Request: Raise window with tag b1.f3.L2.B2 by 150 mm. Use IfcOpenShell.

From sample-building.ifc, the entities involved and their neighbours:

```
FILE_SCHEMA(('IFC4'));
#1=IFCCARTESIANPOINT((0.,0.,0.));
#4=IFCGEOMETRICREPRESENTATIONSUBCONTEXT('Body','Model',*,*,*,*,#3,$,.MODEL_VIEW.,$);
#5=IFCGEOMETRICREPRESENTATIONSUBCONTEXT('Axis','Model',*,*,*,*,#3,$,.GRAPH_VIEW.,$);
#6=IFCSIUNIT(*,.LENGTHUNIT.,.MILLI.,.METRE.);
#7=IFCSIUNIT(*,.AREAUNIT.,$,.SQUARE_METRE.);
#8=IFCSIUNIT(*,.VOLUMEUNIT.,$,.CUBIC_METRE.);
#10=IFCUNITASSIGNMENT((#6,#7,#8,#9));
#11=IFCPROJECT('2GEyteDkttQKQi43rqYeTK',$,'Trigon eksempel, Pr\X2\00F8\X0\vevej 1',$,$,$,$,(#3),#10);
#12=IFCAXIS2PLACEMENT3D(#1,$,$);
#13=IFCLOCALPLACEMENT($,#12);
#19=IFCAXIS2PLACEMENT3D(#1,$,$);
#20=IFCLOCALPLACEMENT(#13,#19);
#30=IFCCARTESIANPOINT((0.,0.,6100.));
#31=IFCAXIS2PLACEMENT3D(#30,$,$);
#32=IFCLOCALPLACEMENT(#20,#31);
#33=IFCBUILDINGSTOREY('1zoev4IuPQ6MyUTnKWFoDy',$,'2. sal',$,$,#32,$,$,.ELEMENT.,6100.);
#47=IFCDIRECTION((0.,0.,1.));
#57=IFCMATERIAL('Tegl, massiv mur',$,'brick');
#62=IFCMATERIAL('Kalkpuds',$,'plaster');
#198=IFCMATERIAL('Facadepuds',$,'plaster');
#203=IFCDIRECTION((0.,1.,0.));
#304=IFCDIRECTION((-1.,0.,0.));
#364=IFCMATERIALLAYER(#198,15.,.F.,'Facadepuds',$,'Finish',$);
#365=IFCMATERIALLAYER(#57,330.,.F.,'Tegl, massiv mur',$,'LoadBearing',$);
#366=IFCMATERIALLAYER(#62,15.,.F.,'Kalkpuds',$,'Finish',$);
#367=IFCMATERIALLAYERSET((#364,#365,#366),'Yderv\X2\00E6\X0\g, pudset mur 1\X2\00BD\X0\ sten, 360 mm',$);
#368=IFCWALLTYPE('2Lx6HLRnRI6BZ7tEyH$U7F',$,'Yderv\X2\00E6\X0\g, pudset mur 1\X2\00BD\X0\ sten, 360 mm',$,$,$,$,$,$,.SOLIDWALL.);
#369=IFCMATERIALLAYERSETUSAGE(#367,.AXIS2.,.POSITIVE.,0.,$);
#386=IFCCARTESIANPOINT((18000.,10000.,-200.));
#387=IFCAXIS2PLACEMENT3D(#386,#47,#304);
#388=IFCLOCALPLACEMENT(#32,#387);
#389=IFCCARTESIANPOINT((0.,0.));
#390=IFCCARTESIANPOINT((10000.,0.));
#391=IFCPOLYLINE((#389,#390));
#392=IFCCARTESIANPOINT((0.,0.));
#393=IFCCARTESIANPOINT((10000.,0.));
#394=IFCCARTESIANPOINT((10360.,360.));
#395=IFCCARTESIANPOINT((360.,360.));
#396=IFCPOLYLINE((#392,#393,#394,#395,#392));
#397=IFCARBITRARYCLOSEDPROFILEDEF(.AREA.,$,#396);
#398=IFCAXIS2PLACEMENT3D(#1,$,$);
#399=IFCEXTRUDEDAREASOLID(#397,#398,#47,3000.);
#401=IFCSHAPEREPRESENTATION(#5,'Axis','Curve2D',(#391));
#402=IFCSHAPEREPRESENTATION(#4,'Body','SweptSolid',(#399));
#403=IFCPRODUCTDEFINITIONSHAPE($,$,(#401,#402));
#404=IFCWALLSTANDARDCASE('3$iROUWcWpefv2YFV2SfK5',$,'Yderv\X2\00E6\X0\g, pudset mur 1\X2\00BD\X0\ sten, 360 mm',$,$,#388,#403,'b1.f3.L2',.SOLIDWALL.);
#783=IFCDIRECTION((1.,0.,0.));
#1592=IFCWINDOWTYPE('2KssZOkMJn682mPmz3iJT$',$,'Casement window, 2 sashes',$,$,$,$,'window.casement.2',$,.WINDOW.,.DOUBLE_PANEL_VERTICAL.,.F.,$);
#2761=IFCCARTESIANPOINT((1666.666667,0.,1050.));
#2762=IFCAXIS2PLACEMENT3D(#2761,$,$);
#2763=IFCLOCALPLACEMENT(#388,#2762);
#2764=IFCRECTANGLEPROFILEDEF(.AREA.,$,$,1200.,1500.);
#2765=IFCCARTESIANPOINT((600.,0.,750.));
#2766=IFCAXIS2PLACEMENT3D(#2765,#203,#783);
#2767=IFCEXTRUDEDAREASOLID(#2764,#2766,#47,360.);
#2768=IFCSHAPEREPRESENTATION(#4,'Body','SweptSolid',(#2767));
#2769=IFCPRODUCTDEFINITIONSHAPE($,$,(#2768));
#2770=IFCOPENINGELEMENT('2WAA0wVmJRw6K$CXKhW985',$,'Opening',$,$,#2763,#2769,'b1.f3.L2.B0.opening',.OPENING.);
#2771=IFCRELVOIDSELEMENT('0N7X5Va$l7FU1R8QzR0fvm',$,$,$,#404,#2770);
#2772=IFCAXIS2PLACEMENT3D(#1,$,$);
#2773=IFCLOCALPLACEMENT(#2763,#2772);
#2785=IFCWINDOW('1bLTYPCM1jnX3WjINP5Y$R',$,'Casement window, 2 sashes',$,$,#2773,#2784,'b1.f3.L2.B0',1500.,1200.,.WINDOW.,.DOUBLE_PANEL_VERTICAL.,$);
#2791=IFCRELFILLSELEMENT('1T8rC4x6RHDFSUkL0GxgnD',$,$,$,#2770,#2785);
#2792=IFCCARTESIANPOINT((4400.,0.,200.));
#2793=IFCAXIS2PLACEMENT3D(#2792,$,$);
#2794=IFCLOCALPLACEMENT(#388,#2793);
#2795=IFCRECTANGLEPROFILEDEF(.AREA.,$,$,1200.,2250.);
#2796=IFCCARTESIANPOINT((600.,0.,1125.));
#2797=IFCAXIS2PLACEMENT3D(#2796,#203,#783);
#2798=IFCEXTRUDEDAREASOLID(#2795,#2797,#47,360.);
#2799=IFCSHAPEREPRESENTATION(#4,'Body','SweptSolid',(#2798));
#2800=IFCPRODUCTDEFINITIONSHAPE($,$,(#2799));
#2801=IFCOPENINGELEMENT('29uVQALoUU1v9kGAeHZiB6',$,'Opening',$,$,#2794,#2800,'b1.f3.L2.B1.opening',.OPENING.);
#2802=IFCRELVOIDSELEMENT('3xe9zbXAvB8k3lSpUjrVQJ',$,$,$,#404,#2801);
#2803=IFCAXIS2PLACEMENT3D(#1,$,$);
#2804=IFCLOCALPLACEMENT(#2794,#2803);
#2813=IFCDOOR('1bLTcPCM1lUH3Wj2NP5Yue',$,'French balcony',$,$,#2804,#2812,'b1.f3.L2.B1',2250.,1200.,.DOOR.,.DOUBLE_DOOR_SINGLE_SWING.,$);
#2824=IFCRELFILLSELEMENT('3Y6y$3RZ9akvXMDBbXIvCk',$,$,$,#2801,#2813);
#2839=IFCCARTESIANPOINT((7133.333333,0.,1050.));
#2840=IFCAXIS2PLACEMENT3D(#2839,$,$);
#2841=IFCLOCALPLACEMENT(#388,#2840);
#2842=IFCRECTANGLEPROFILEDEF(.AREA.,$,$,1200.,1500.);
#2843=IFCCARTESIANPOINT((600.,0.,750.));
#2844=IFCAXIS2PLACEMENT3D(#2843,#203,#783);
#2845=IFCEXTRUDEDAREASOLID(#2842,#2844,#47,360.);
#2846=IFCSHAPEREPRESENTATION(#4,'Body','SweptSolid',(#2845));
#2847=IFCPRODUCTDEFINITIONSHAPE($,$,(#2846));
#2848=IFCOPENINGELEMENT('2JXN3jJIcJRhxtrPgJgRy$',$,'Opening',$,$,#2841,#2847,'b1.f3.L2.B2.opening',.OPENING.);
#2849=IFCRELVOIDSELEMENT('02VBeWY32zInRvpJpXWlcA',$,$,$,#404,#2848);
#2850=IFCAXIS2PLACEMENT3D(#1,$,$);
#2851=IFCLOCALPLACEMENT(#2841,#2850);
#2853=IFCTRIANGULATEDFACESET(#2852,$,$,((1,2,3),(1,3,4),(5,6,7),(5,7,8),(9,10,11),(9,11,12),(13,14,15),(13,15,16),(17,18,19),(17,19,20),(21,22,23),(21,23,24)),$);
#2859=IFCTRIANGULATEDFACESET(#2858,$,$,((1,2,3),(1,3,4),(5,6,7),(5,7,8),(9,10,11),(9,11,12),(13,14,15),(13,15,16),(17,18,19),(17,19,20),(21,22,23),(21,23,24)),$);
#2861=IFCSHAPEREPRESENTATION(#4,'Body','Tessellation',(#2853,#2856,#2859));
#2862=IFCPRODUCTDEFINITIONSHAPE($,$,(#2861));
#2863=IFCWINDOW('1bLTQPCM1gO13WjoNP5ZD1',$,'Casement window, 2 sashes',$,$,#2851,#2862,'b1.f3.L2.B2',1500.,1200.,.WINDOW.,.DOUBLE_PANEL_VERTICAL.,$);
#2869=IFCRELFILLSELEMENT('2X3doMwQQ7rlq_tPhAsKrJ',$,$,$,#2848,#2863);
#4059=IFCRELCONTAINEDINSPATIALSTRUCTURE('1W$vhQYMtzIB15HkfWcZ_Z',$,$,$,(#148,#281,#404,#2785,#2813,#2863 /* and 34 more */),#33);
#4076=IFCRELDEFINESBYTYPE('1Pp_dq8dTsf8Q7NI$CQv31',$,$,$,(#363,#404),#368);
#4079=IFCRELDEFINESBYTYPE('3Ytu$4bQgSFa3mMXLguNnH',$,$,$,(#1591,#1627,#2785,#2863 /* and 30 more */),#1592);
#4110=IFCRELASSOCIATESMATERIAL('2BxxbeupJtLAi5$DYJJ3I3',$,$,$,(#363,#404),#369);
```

```python
import numpy as np
import ifcopenshell
import ifcopenshell.api.geometry
import ifcopenshell.util.placement
import ifcopenshell.util.unit

model = ifcopenshell.open("sample-building.ifc")
unit_scale = ifcopenshell.util.unit.calculate_unit_scale(model)

window = model.by_guid("1bLTQPCM1gO13WjoNP5ZD1")
opening = window.FillsVoids[0].RelatingOpeningElement
dz = 150.0

shift = np.array([0.0, 0.0, dz])
# The window is placed relative to its opening, so it follows when the opening moves.
matrix = ifcopenshell.util.placement.get_local_placement(opening.ObjectPlacement)
matrix[:3, 3] += shift
ifcopenshell.api.geometry.edit_object_placement(
    model, product=opening, matrix=matrix, is_si=False, should_transform_children=True
)

print(f"moved by {dz * unit_scale:+.3f} m")

model.write("sample-building_updated.ifc")
```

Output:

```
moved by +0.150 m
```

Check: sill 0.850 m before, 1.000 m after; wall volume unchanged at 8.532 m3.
